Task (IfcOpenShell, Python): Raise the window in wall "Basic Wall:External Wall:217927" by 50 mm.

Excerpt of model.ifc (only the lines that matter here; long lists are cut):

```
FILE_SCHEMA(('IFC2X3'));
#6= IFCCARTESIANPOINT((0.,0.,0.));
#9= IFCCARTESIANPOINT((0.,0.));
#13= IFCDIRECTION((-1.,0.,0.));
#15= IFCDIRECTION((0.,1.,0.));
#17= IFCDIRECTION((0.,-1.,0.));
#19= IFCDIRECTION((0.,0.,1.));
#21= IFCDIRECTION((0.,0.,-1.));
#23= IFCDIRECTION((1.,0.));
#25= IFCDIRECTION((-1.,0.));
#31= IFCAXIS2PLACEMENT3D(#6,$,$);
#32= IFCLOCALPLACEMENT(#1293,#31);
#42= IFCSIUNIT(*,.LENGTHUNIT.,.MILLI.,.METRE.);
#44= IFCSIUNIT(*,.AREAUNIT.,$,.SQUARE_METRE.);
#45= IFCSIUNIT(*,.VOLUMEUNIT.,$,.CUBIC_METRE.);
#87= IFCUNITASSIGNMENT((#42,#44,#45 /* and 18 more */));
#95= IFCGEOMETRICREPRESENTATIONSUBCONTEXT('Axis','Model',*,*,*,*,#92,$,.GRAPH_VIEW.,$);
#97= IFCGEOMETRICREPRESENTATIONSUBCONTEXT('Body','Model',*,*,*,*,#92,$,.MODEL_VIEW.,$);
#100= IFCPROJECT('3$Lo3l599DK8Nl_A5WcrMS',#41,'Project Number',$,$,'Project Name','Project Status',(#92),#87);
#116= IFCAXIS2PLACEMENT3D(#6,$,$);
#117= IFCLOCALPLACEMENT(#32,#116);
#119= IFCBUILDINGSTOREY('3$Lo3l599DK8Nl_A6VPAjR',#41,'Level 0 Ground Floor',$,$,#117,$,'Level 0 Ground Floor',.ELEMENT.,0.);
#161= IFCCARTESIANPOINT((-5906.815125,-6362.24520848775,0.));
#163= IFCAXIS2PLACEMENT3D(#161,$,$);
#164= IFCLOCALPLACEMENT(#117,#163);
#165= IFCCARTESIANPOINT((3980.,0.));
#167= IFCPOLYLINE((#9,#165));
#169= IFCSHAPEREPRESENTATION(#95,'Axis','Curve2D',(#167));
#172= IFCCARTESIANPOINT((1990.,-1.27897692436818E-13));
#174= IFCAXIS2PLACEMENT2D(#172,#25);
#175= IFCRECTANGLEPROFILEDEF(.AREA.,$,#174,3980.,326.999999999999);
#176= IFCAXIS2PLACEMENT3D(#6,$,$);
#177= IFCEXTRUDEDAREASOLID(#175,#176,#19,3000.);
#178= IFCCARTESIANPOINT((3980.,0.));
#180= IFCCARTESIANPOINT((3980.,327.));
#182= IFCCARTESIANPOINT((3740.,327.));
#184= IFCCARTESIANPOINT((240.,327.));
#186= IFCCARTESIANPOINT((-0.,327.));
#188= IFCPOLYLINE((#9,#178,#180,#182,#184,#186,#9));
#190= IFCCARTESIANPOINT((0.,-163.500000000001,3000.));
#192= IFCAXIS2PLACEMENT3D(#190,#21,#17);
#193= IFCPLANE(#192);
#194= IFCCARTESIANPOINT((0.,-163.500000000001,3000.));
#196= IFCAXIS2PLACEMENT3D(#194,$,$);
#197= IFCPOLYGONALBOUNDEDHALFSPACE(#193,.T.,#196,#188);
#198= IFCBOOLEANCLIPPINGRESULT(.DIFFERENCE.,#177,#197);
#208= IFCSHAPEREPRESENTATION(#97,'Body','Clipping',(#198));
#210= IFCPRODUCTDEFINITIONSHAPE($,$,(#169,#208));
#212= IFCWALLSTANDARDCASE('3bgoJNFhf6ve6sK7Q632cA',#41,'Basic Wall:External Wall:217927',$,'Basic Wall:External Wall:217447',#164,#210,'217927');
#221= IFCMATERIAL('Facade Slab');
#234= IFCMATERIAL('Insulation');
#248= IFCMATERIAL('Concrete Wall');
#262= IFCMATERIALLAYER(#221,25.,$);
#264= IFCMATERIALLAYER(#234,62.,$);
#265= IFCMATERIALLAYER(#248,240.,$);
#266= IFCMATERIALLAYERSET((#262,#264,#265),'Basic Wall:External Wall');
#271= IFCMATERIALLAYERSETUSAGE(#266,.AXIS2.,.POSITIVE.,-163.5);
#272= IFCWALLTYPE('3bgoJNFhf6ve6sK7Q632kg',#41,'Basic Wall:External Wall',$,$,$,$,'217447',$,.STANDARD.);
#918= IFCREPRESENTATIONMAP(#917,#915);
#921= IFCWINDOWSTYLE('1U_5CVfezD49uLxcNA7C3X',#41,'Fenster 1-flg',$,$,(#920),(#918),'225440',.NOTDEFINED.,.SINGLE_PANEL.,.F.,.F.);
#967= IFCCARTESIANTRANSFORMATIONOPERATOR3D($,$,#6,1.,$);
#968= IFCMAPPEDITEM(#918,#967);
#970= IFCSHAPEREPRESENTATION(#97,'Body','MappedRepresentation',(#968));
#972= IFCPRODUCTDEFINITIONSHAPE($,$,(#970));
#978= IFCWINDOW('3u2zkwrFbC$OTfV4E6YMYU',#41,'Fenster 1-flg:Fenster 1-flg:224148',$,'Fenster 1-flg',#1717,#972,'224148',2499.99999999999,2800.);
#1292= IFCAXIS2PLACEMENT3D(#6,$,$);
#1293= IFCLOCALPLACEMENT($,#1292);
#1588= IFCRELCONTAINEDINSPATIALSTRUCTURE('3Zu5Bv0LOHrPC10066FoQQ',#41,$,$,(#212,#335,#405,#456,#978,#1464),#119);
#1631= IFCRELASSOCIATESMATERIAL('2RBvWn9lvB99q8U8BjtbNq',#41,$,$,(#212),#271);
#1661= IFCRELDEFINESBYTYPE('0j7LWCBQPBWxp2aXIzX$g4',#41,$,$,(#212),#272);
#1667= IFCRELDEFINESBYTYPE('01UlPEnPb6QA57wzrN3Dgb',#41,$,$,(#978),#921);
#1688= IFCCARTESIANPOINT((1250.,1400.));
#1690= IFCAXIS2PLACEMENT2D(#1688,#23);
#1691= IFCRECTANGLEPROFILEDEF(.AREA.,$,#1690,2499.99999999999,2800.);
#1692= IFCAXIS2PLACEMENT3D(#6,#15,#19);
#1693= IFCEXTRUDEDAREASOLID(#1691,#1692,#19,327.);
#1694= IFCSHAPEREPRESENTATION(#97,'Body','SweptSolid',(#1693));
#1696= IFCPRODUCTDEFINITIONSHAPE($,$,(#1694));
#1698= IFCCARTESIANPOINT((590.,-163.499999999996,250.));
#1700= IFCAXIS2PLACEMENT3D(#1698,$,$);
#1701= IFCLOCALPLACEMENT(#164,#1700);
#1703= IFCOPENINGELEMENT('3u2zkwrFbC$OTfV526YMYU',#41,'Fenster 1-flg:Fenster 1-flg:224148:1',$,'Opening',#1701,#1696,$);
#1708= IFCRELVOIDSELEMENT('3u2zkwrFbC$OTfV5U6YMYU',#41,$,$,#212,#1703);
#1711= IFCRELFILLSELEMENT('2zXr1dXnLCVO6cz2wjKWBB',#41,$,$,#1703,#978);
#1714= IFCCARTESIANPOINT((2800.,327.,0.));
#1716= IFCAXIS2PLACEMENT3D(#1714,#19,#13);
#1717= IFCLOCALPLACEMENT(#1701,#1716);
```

```python
import numpy as np
import ifcopenshell
import ifcopenshell.api.geometry
import ifcopenshell.util.placement
import ifcopenshell.util.unit

model = ifcopenshell.open("model.ifc")
unit_scale = ifcopenshell.util.unit.calculate_unit_scale(model)

window = model.by_id(978)
opening = window.FillsVoids[0].RelatingOpeningElement
dz = 0.05 / unit_scale

shift = np.array([0.0, 0.0, dz])
# The window is placed relative to its opening, so it follows when the opening moves.
matrix = ifcopenshell.util.placement.get_local_placement(opening.ObjectPlacement)
matrix[:3, 3] += shift
ifcopenshell.api.geometry.edit_object_placement(
    model, product=opening, matrix=matrix, is_si=False, should_transform_children=True
)

print(f"moved by {dz * unit_scale:+.3f} m")

model.write("model_updated.ifc")
```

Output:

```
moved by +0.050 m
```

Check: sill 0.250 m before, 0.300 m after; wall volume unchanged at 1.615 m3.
